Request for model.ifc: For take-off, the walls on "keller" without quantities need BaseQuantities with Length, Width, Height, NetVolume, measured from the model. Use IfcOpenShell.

First a look at what the model holds.

```python
import ifcopenshell
import ifcopenshell.util.element
import ifcopenshell.util.unit

model = ifcopenshell.open("model.ifc")
print(model.schema)
for unit_type in ("LENGTHUNIT", "AREAUNIT", "VOLUMEUNIT"):
    print(unit_type, ifcopenshell.util.unit.calculate_unit_scale(model, unit_type))
storey = next(s for s in model.by_type("IfcBuildingStorey") if s.Name == "keller")
walls = [e for e in ifcopenshell.util.element.get_decomposition(storey) if e.is_a("IfcWall")]
for e in sorted(walls, key=lambda e: e.id()):
    print(e.id(), e.is_a(), e.Name, list(ifcopenshell.util.element.get_psets(e, qtos_only=True)), sep=" | ")
```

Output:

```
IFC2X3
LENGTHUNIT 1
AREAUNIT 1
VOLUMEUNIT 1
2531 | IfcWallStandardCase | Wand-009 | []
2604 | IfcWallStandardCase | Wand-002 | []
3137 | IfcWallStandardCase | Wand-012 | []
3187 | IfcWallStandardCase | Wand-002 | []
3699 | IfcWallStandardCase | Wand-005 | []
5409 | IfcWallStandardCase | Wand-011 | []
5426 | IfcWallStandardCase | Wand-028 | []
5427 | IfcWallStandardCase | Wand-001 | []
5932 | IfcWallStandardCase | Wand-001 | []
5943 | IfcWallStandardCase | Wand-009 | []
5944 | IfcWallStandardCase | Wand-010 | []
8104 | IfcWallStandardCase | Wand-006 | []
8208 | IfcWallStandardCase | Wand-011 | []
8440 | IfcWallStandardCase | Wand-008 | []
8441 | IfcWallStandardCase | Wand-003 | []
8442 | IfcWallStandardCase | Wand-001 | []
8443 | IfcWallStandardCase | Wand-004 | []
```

```python
import ifcopenshell
import ifcopenshell.api.pset
import ifcopenshell.geom
import ifcopenshell.util.element
import ifcopenshell.util.shape
import ifcopenshell.util.unit

model = ifcopenshell.open("model.ifc")
unit_scale = ifcopenshell.util.unit.calculate_unit_scale(model)
volume_scale = ifcopenshell.util.unit.calculate_unit_scale(model, "VOLUMEUNIT")
settings = ifcopenshell.geom.settings()

storey = next(s for s in model.by_type("IfcBuildingStorey") if s.Name == "keller")
walls = [e for e in ifcopenshell.util.element.get_decomposition(storey) if e.is_a("IfcWall")]

for e in sorted(walls, key=lambda e: e.id()):
    if ifcopenshell.util.element.get_psets(e, qtos_only=True, should_inherit=False):
        continue
    # Geometry comes back in metres, in the element's own axes.
    shape = ifcopenshell.geom.create_shape(settings, e)
    values = {
        "Length": ifcopenshell.util.shape.get_x(shape.geometry) / unit_scale,
        "Width": ifcopenshell.util.shape.get_y(shape.geometry) / unit_scale,
        "Height": ifcopenshell.util.shape.get_z(shape.geometry) / unit_scale,
        "NetVolume": ifcopenshell.util.shape.get_volume(shape.geometry) / volume_scale,
    }
    qto = ifcopenshell.api.pset.add_qto(model, product=e, name="BaseQuantities")
    ifcopenshell.api.pset.edit_qto(model, qto=qto, properties=values)
    print(e.id(), {k: round(v, 3) for k, v in values.items()})

model.write("model_updated.ifc")
```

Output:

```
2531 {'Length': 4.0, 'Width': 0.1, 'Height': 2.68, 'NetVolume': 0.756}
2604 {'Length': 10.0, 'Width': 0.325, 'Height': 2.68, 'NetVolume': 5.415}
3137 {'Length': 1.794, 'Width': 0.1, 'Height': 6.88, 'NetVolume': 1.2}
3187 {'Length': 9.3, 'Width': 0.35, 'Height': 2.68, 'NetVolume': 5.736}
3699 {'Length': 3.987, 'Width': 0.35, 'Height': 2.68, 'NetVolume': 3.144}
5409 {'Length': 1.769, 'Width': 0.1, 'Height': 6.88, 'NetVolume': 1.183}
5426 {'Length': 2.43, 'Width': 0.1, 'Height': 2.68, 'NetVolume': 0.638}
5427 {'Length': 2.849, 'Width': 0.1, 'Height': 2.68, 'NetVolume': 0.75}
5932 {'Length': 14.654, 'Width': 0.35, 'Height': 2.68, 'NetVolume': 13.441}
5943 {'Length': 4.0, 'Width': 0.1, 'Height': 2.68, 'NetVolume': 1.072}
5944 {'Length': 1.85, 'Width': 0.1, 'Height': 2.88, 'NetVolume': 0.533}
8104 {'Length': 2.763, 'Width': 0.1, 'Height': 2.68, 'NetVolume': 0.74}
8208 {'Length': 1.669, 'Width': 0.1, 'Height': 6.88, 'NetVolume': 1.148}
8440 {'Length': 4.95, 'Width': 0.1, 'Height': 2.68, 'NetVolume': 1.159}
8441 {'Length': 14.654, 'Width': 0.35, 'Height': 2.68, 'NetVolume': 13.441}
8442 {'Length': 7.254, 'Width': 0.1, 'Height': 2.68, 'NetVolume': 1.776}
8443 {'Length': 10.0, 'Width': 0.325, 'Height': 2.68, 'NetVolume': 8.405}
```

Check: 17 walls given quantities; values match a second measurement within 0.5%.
